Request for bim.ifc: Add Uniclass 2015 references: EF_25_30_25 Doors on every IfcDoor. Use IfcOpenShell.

First a look at what the model holds.

```python
import ifcopenshell

model = ifcopenshell.open("bim.ifc")
print(model.schema)
print("classifications:", [c.Name for c in model.by_type("IfcClassification")])
for ifc_class in ("IfcDoor", "IfcRoof", "IfcStair", "IfcWall", "IfcWindow"):
    print(ifc_class, len(model.by_type(ifc_class)))
```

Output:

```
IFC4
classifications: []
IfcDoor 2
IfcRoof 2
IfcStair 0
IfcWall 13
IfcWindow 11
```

```python
import ifcopenshell
import ifcopenshell.api.classification

model = ifcopenshell.open("bim.ifc")

system = ifcopenshell.api.classification.add_classification(model, classification="Uniclass 2015")

codes = {
    "IfcDoor": ("EF_25_30_25", "Doors"),
}
for ifc_class, (code, name) in codes.items():
    products = model.by_type(ifc_class)
    ifcopenshell.api.classification.add_reference(
        model, products=products, classification=system, identification=code, name=name
    )
    print(code, len(products))

model.write("bim_edited.ifc")
```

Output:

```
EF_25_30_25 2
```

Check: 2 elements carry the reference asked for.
